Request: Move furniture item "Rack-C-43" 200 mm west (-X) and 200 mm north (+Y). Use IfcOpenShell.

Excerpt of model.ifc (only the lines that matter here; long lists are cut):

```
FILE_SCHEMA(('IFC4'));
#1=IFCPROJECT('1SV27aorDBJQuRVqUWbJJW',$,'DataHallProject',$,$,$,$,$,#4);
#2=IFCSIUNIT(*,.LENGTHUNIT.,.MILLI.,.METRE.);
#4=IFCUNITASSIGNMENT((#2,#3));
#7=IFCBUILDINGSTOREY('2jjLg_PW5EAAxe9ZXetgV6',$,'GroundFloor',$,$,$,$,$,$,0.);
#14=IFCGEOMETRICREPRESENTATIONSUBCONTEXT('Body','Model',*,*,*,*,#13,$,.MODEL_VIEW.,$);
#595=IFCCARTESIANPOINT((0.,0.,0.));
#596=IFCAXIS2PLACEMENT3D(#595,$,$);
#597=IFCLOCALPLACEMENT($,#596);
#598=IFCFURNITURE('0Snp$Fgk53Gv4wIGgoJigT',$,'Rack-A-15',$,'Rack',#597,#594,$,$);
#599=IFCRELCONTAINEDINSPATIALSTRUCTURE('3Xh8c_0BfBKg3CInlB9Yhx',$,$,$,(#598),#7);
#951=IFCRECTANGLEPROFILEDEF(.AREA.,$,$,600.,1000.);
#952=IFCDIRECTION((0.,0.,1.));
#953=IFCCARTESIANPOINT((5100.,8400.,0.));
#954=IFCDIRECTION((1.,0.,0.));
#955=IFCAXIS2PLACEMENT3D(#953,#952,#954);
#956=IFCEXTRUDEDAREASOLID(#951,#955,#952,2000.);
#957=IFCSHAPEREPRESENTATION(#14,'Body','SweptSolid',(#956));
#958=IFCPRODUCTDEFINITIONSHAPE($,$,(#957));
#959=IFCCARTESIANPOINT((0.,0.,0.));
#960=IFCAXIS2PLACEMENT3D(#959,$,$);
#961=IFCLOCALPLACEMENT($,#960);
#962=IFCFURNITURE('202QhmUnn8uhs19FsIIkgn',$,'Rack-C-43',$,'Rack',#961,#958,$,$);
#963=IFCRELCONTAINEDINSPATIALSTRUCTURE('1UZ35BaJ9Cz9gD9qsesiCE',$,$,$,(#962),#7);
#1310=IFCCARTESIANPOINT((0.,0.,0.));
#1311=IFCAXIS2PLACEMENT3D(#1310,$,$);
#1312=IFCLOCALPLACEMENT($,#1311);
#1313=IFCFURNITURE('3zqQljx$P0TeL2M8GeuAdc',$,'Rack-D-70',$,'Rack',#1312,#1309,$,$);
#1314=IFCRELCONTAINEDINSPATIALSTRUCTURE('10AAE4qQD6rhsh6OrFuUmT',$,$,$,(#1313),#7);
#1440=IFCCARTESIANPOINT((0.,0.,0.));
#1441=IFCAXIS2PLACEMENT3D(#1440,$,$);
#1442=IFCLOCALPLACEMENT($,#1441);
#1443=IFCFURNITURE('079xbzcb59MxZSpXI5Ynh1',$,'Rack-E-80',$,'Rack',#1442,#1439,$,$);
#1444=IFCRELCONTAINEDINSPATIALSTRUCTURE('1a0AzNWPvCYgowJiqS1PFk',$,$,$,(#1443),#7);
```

```python
import ifcopenshell
import ifcopenshell.api.geometry
import ifcopenshell.util.placement

model = ifcopenshell.open("model.ifc")

item = model.by_guid("202QhmUnn8uhs19FsIIkgn")
matrix = ifcopenshell.util.placement.get_local_placement(item.ObjectPlacement)
matrix[0, 3] -= 200.0
matrix[1, 3] += 200.0
ifcopenshell.api.geometry.edit_object_placement(model, product=item, matrix=matrix, is_si=False)

print(ifcopenshell.util.placement.get_local_placement(item.ObjectPlacement).round(3) + 0.0)

model.write("model-out.ifc")
```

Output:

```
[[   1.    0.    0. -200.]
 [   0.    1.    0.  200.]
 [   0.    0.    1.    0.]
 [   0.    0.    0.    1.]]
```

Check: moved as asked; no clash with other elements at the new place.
